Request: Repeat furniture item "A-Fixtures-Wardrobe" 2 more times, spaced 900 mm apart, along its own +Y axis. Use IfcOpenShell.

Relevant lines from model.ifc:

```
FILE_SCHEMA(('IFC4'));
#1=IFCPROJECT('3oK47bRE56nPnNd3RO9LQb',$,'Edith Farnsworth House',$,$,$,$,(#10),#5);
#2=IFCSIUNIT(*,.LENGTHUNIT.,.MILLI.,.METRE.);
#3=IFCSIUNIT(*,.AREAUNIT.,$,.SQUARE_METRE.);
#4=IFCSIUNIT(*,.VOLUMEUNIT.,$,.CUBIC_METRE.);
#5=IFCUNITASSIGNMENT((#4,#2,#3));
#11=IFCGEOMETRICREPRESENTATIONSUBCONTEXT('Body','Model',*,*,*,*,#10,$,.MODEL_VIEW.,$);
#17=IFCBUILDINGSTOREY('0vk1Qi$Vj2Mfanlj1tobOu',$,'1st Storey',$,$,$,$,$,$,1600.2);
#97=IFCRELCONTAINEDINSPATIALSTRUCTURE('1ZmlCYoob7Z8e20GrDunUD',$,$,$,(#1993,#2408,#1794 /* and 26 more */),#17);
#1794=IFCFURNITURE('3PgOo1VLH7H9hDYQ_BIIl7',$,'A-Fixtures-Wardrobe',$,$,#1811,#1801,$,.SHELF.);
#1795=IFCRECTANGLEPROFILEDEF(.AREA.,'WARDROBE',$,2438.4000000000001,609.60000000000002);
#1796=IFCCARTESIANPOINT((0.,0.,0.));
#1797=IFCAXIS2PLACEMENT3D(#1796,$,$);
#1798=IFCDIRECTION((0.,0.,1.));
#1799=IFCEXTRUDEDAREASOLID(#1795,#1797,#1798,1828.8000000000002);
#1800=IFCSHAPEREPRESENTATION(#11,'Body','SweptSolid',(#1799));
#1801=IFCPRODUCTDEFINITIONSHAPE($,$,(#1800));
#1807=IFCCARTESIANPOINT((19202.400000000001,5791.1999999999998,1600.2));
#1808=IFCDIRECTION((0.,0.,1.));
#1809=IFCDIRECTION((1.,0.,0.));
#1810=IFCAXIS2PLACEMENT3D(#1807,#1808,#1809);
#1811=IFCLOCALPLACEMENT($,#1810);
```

```python
import ifcopenshell
import ifcopenshell.api.geometry
import ifcopenshell.api.root
import ifcopenshell.util.element
import ifcopenshell.util.placement
import ifcopenshell.util.unit

model = ifcopenshell.open("model.ifc")
unit_scale = ifcopenshell.util.unit.calculate_unit_scale(model)

source = model.by_id(1794)
base = ifcopenshell.util.placement.get_local_placement(source.ObjectPlacement)
step = base[:3, 1] * 0.9 / unit_scale

for i in range(1, 3):
    copy = ifcopenshell.api.root.copy_class(model, product=source)
    copy.Representation = ifcopenshell.util.element.copy_deep(
        model, source.Representation, exclude=["IfcGeometricRepresentationContext", "IfcRepresentationMap"]
    )
    matrix = base.copy()
    matrix[:3, 3] += i * step
    print("added at", matrix[:3, 3].round(3) + 0.0)
    ifcopenshell.api.geometry.edit_object_placement(model, product=copy, matrix=matrix, is_si=False)

model.write("model_v2.ifc")
```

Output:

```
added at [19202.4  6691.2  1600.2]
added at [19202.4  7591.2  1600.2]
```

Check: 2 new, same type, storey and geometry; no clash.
